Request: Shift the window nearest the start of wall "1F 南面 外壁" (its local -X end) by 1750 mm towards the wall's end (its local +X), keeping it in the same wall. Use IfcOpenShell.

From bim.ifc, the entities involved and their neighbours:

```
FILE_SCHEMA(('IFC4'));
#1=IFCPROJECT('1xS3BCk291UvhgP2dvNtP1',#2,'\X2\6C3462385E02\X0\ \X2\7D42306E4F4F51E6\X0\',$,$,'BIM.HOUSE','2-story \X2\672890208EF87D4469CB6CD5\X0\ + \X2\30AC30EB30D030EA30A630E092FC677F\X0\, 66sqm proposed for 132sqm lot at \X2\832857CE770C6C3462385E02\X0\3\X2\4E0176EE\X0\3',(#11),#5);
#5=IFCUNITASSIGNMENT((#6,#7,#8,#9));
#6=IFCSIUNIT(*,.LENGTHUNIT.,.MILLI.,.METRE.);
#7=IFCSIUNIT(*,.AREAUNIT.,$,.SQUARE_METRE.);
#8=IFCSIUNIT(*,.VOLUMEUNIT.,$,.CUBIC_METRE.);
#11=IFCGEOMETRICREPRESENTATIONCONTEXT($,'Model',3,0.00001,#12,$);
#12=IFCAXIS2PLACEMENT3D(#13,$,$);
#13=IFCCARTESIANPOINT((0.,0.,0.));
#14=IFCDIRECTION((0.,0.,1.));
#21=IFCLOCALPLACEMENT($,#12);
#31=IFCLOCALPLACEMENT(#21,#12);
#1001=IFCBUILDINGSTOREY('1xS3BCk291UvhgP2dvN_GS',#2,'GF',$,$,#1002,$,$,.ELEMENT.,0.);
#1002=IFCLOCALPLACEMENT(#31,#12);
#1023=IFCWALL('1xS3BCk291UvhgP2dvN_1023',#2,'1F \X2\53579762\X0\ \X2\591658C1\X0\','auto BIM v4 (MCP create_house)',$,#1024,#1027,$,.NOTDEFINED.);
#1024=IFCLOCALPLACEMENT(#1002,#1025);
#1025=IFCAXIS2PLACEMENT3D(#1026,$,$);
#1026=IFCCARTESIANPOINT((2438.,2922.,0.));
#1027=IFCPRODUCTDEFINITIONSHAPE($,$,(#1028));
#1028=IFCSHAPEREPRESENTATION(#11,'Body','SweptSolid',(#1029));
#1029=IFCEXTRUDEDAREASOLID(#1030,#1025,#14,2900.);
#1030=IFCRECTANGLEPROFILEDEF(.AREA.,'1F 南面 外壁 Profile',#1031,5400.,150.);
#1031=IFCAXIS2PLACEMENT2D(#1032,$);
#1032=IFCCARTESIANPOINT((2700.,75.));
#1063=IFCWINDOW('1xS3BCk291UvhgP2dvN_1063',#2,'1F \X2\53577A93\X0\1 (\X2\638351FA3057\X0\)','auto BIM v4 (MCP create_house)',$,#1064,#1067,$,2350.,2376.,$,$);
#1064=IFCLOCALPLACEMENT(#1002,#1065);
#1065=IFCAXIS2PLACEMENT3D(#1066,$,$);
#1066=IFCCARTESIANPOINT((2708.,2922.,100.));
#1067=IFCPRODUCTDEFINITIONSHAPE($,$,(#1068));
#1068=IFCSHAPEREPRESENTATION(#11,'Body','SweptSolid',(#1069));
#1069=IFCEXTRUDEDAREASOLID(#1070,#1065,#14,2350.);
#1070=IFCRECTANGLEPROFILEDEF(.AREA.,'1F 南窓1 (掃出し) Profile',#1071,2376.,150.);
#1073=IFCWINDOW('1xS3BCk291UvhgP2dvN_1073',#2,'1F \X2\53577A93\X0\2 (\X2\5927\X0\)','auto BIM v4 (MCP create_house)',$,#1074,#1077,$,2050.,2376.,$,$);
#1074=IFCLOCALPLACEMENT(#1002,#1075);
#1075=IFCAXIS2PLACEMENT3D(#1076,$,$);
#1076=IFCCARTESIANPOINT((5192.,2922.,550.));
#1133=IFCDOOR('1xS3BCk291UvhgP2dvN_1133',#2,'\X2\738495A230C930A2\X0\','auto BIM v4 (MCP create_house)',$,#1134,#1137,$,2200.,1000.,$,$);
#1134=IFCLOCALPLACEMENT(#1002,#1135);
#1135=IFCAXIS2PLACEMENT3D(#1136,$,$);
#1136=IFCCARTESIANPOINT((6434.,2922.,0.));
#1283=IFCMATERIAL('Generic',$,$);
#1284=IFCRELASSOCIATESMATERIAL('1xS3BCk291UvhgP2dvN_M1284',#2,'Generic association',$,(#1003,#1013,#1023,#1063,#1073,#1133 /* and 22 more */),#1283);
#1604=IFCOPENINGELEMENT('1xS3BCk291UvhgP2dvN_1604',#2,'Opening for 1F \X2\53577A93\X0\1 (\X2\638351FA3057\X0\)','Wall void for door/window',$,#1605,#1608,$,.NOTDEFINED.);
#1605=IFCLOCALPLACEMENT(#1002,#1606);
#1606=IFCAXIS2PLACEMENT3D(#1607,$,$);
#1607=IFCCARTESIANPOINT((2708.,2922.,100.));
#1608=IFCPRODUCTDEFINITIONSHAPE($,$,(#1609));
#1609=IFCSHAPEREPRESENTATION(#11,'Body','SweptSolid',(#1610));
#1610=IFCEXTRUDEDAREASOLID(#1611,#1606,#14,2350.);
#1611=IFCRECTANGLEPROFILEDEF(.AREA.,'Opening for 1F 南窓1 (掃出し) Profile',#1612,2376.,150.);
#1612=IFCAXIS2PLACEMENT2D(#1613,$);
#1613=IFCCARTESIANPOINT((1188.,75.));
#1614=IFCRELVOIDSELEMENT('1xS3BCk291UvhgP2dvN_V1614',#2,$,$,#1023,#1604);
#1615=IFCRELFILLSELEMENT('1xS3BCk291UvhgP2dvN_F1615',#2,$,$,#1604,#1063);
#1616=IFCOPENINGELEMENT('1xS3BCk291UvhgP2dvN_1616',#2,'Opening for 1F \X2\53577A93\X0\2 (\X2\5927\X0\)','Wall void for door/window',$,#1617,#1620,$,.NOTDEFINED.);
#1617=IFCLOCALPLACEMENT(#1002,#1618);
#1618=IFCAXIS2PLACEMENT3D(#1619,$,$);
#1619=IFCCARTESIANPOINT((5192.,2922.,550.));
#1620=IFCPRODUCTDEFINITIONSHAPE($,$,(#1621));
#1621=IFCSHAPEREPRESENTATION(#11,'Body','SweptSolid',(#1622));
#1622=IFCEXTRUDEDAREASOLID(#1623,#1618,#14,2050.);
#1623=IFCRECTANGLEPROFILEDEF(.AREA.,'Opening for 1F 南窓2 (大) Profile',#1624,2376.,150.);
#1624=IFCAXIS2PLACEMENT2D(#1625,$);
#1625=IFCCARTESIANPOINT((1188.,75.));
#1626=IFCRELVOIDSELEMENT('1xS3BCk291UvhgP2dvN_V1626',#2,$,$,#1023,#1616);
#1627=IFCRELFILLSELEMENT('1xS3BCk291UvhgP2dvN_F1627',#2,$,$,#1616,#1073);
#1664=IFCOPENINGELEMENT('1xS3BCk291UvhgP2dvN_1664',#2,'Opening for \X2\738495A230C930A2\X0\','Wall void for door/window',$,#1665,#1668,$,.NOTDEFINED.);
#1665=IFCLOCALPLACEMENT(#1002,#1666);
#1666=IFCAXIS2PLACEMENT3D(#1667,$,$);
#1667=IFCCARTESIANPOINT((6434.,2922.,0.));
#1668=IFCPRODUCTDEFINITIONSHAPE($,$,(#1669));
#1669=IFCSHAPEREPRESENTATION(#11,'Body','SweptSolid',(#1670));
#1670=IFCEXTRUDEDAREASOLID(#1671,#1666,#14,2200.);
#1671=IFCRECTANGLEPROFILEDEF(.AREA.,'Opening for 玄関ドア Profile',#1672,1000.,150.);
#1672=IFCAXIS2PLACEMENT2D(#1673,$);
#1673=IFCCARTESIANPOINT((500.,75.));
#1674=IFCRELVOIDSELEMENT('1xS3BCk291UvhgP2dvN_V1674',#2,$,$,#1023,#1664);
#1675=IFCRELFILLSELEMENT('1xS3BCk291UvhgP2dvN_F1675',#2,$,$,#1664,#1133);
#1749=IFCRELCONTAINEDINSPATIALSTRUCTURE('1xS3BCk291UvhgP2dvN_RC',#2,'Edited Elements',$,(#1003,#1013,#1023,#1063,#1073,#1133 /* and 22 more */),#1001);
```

```python
import ifcopenshell
import ifcopenshell.api.geometry
import ifcopenshell.util.placement
import ifcopenshell.util.unit

model = ifcopenshell.open("bim.ifc")
unit_scale = ifcopenshell.util.unit.calculate_unit_scale(model)

window = model.by_id(1063)
opening = window.FillsVoids[0].RelatingOpeningElement
wall = opening.VoidsElements[0].RelatingBuildingElement

wall_matrix = ifcopenshell.util.placement.get_local_placement(wall.ObjectPlacement)
shift = wall_matrix[:3, 0] * 1.75 / unit_scale
before = ifcopenshell.util.placement.get_local_placement(window.ObjectPlacement)[:3, 3].copy()

# The window is not placed relative to its opening, so move both.
for product in (opening, window):
    matrix = ifcopenshell.util.placement.get_local_placement(product.ObjectPlacement)
    matrix[:3, 3] += shift
    ifcopenshell.api.geometry.edit_object_placement(model, product=product, matrix=matrix, is_si=False)

after = ifcopenshell.util.placement.get_local_placement(window.ObjectPlacement)[:3, 3]
print("window moved by", (after - before).round(3) + 0.0)

model.write("bim-out.ifc")
```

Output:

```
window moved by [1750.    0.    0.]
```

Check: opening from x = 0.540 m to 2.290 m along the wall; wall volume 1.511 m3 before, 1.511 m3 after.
